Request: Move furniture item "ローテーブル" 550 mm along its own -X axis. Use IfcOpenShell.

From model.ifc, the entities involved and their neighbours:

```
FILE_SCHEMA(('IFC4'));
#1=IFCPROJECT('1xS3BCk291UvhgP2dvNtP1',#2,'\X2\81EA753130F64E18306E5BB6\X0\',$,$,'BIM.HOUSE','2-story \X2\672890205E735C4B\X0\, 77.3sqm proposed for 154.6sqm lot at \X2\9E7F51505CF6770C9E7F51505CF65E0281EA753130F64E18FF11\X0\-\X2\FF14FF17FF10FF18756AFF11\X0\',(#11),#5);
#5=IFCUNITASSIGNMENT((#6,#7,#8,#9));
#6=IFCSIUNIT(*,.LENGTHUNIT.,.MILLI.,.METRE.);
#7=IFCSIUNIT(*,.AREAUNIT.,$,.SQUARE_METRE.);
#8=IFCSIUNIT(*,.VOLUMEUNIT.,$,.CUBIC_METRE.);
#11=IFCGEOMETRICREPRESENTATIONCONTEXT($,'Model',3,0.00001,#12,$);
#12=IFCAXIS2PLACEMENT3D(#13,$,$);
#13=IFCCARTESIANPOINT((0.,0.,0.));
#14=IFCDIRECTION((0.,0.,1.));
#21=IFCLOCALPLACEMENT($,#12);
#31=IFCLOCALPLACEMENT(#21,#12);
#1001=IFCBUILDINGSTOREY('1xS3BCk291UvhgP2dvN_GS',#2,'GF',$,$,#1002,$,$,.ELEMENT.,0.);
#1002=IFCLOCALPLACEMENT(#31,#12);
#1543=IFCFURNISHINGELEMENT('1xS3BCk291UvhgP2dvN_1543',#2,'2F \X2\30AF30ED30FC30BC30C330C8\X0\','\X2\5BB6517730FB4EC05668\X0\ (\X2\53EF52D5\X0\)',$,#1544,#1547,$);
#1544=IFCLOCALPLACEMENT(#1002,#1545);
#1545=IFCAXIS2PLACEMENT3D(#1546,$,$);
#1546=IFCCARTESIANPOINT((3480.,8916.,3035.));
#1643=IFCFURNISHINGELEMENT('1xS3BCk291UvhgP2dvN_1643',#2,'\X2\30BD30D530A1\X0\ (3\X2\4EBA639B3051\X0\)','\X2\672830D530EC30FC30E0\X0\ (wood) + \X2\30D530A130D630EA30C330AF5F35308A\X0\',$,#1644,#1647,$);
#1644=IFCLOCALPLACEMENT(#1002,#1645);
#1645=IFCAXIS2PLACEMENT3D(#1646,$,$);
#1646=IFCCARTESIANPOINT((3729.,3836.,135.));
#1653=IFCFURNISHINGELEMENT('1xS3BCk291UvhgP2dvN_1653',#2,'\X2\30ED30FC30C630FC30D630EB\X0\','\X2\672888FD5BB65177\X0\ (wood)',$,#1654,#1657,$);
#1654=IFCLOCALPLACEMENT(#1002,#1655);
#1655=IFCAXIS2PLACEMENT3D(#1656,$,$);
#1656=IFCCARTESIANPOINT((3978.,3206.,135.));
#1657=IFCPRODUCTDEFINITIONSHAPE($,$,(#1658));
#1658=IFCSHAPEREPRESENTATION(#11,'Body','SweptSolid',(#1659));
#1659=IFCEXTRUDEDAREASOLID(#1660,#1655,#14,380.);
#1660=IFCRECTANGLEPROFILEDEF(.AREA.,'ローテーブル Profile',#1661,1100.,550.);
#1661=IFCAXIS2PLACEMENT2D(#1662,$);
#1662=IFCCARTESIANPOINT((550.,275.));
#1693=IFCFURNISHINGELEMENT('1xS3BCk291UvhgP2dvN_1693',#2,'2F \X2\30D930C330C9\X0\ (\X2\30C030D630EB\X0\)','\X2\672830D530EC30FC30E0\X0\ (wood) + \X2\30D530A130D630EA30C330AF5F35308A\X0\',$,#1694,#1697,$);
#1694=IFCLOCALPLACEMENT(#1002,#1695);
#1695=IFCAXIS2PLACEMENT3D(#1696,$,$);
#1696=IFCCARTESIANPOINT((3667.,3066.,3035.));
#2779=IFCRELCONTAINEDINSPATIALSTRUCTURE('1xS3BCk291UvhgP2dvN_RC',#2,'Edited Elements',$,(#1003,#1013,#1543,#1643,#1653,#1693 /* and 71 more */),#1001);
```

```python
import ifcopenshell
import ifcopenshell.api.geometry
import ifcopenshell.util.placement
import ifcopenshell.util.unit

model = ifcopenshell.open("model.ifc")
unit_scale = ifcopenshell.util.unit.calculate_unit_scale(model)

item = model.by_guid("1xS3BCk291UvhgP2dvN_1653")
matrix = ifcopenshell.util.placement.get_local_placement(item.ObjectPlacement)
matrix[:3, 3] -= matrix[:3, 0] * 0.55 / unit_scale
ifcopenshell.api.geometry.edit_object_placement(model, product=item, matrix=matrix, is_si=False)

print(ifcopenshell.util.placement.get_local_placement(item.ObjectPlacement).round(3) + 0.0)

model.write("model_edited.ifc")
```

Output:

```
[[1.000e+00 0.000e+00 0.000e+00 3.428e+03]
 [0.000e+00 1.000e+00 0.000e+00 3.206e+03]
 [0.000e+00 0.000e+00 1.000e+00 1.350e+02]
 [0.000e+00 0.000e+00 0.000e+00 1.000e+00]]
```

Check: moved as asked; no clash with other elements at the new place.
